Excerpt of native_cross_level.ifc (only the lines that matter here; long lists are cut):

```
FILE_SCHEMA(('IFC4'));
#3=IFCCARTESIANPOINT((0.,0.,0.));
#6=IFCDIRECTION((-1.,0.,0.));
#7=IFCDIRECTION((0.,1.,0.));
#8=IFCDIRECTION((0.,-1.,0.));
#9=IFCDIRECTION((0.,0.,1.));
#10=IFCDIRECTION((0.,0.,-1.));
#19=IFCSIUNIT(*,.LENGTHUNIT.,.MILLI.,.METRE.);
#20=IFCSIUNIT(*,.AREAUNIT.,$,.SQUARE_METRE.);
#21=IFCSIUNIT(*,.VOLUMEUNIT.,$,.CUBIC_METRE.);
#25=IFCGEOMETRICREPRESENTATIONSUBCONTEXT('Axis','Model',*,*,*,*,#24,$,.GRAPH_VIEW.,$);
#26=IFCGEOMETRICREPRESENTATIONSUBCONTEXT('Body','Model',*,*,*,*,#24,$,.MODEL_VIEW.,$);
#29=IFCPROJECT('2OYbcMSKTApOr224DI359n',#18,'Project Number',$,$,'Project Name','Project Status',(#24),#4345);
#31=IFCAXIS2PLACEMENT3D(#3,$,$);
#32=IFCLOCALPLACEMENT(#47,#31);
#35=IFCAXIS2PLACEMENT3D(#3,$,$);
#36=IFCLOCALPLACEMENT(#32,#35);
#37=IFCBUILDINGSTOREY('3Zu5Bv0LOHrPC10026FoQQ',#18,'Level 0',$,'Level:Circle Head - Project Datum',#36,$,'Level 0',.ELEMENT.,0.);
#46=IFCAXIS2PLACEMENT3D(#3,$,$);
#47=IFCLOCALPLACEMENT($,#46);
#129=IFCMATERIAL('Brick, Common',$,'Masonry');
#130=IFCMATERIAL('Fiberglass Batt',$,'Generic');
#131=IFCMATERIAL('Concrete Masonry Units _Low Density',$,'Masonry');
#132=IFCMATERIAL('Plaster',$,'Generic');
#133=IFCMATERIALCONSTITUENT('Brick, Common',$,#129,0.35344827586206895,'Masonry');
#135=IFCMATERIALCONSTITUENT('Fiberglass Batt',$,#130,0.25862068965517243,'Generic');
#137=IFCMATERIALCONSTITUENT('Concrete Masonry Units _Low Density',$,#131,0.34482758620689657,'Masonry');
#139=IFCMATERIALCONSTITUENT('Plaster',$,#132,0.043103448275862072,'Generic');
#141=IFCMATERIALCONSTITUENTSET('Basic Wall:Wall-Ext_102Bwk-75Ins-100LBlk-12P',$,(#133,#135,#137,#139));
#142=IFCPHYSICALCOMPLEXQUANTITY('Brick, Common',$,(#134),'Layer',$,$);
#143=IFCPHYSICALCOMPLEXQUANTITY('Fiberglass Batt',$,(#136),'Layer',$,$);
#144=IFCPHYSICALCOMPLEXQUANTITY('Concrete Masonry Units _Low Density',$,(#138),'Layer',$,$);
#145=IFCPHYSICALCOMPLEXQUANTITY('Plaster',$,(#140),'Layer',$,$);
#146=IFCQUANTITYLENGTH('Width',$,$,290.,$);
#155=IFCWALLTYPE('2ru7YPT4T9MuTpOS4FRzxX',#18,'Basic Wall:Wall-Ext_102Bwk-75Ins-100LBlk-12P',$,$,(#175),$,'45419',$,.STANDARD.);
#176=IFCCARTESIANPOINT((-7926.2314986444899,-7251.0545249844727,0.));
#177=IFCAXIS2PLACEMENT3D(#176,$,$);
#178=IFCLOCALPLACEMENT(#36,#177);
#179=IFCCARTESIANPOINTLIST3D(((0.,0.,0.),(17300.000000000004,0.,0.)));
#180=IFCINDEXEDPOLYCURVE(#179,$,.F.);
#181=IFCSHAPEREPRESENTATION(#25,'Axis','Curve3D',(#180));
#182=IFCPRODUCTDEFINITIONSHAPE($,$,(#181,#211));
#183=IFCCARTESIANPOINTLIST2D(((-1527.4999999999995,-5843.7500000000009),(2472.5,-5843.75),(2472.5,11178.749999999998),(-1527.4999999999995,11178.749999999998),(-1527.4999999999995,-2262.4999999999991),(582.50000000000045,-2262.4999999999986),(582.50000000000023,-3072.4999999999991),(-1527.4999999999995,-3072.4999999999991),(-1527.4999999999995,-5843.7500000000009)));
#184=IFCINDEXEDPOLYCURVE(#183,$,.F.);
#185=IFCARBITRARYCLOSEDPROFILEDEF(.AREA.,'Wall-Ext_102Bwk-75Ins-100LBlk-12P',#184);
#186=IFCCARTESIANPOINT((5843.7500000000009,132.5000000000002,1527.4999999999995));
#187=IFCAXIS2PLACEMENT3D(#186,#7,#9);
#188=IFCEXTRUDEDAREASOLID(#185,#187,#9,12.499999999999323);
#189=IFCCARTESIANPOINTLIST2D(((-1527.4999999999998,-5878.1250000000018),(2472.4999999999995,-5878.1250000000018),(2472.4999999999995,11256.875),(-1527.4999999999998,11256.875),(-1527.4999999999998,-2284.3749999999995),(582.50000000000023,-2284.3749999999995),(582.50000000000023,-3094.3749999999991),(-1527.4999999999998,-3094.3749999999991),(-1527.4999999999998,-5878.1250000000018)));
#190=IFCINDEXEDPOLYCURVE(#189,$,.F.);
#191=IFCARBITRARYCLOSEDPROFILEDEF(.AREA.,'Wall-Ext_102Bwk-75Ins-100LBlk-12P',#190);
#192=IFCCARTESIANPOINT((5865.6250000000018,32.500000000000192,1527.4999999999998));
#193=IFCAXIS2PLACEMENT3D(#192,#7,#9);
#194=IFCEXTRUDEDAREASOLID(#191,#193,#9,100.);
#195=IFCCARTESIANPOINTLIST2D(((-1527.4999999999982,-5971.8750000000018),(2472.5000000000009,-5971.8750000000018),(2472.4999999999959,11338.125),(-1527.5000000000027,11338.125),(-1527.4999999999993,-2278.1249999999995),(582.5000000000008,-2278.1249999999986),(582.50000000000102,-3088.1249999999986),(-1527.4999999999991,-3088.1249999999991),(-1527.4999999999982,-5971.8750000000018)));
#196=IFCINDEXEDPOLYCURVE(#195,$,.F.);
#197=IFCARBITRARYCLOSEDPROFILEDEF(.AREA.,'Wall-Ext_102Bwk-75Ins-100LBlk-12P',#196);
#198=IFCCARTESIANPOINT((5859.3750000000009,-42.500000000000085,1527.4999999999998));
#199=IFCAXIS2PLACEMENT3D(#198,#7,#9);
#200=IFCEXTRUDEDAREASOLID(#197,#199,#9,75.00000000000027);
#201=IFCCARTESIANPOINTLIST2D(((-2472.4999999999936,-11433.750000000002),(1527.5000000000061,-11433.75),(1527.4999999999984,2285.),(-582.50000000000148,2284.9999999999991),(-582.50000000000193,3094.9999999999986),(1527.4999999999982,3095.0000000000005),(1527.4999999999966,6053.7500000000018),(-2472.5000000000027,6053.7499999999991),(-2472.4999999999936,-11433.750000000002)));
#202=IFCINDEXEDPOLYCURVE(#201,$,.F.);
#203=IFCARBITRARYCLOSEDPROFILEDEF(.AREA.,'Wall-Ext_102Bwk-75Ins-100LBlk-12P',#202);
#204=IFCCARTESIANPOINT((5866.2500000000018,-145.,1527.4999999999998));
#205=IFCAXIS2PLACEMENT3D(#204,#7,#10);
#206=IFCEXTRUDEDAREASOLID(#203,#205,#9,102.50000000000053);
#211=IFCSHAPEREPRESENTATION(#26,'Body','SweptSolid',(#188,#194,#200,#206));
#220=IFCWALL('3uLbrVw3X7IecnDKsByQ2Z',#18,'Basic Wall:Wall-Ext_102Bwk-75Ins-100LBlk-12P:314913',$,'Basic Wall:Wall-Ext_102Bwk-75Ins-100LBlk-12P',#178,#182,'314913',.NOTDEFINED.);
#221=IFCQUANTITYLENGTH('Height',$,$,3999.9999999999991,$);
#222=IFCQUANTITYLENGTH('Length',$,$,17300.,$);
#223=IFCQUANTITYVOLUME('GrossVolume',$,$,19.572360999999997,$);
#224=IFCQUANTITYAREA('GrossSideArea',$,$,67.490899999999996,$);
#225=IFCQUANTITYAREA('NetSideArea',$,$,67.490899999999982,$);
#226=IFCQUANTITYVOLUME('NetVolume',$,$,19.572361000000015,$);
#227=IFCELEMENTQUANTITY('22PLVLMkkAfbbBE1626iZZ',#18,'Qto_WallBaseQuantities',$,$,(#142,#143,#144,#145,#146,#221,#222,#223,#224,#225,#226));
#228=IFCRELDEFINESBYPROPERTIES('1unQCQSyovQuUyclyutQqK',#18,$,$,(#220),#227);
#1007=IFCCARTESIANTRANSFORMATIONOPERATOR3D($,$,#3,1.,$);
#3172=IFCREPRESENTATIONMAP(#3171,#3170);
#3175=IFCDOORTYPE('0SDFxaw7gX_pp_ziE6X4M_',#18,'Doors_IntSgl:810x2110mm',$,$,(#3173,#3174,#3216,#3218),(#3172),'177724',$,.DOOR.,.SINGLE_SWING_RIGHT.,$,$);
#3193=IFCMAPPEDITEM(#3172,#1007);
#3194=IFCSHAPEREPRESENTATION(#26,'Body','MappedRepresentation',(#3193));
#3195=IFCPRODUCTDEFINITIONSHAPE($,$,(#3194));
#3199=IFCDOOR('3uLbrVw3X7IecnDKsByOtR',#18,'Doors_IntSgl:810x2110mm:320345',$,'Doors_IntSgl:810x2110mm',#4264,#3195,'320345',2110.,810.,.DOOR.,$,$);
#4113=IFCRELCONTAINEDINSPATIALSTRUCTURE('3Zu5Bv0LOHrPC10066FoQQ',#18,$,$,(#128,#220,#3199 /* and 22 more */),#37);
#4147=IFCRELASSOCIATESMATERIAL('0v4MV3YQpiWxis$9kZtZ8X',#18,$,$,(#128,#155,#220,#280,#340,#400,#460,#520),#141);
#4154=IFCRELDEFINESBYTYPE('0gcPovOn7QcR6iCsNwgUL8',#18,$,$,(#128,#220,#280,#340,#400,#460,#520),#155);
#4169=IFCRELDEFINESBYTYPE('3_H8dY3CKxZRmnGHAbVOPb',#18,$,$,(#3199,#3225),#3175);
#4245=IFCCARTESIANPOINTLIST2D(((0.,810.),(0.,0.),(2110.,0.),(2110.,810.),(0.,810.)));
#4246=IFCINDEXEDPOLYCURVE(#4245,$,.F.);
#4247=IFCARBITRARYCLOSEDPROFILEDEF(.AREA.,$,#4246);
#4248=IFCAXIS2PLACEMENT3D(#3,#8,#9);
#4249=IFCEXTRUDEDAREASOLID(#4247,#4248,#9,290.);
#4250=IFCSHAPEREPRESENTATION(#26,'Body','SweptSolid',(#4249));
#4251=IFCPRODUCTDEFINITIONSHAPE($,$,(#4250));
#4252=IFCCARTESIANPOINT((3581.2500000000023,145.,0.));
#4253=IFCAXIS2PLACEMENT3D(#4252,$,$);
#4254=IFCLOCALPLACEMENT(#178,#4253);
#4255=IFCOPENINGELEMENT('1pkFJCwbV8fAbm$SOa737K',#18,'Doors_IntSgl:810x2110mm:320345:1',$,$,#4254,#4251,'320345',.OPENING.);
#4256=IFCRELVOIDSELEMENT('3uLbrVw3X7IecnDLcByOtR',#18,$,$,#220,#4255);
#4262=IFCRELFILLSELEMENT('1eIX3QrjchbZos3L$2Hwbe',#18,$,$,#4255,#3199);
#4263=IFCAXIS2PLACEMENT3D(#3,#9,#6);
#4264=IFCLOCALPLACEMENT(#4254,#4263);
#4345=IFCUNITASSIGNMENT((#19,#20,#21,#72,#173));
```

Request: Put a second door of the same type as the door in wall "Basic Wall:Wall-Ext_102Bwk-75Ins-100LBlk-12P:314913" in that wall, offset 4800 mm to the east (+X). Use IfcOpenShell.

```python
import ifcopenshell
import ifcopenshell.api.feature
import ifcopenshell.api.geometry
import ifcopenshell.api.pset
import ifcopenshell.api.root
import ifcopenshell.geom
import ifcopenshell.util.element
import ifcopenshell.util.placement
import ifcopenshell.util.shape
import ifcopenshell.util.unit

model = ifcopenshell.open("native_cross_level.ifc")
unit_scale = ifcopenshell.util.unit.calculate_unit_scale(model)
area_scale = ifcopenshell.util.unit.calculate_unit_scale(model, "AREAUNIT")
volume_scale = ifcopenshell.util.unit.calculate_unit_scale(model, "VOLUMEUNIT")
settings = ifcopenshell.geom.settings()


def volume(element):
    """Net volume in cubic metres, openings subtracted."""
    shape = ifcopenshell.geom.create_shape(settings, element)
    return ifcopenshell.util.shape.get_volume(shape.geometry)


def reuse_history(source, copy):
    """copy_class also copies each property set's owner history, people and application; keep the originals."""
    for rel in copy.IsDefinedBy:
        if rel.is_a("IfcRelDefinesByProperties") and (history := rel.RelatingPropertyDefinition.OwnerHistory):
            rel.RelatingPropertyDefinition.OwnerHistory = source.OwnerHistory
            ifcopenshell.util.element.remove_deep2(model, history)


door = model.by_guid("3uLbrVw3X7IecnDKsByOtR")
opening = door.FillsVoids[0].RelatingOpeningElement
wall = opening.VoidsElements[0].RelatingBuildingElement
before = volume(wall)
shift = ifcopenshell.util.placement.get_local_placement(wall.ObjectPlacement)[:3, 0] * 4.8 / unit_scale

# copy_class copies the void relationship, type, container and properties, but no geometry.
new_opening = ifcopenshell.api.root.copy_class(model, product=opening)
new_opening.Representation = ifcopenshell.util.element.copy_deep(
    model, opening.Representation, exclude=["IfcGeometricRepresentationContext", "IfcRepresentationMap"]
)
new_opening.Name = "Doors_IntSgl:810x2110mm"
new_opening.Tag = None
reuse_history(opening, new_opening)
new_door = ifcopenshell.api.root.copy_class(model, product=door)
new_door.Representation = ifcopenshell.util.element.copy_deep(
    model, door.Representation, exclude=["IfcGeometricRepresentationContext", "IfcRepresentationMap"]
)
new_door.Name = "Doors_IntSgl:810x2110mm"
new_door.Tag = None
reuse_history(door, new_door)
ifcopenshell.api.feature.add_filling(model, opening=new_opening, element=new_door)

for old, new in ((opening, new_opening), (door, new_door)):
    matrix = ifcopenshell.util.placement.get_local_placement(old.ObjectPlacement)
    matrix[:3, 3] += shift
    ifcopenshell.api.geometry.edit_object_placement(model, product=new, matrix=matrix, is_si=False)

after = volume(wall)
thickness = 0.29  # wall thickness in metres

# Update the wall's stored quantities.
qto = model.by_id(ifcopenshell.util.element.get_pset(wall, "Qto_WallBaseQuantities", should_inherit=False)["id"])
ifcopenshell.api.pset.edit_qto(model, qto=qto, properties={
    "NetSideArea": after / thickness / area_scale,
    "NetVolume": after / volume_scale,
})

print(f"wall volume {before:.3f} -> {after:.3f} m3")

model.write("native_cross_level-out.ifc")
```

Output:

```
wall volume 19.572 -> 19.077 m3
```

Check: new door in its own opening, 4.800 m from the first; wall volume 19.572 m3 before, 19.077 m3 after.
